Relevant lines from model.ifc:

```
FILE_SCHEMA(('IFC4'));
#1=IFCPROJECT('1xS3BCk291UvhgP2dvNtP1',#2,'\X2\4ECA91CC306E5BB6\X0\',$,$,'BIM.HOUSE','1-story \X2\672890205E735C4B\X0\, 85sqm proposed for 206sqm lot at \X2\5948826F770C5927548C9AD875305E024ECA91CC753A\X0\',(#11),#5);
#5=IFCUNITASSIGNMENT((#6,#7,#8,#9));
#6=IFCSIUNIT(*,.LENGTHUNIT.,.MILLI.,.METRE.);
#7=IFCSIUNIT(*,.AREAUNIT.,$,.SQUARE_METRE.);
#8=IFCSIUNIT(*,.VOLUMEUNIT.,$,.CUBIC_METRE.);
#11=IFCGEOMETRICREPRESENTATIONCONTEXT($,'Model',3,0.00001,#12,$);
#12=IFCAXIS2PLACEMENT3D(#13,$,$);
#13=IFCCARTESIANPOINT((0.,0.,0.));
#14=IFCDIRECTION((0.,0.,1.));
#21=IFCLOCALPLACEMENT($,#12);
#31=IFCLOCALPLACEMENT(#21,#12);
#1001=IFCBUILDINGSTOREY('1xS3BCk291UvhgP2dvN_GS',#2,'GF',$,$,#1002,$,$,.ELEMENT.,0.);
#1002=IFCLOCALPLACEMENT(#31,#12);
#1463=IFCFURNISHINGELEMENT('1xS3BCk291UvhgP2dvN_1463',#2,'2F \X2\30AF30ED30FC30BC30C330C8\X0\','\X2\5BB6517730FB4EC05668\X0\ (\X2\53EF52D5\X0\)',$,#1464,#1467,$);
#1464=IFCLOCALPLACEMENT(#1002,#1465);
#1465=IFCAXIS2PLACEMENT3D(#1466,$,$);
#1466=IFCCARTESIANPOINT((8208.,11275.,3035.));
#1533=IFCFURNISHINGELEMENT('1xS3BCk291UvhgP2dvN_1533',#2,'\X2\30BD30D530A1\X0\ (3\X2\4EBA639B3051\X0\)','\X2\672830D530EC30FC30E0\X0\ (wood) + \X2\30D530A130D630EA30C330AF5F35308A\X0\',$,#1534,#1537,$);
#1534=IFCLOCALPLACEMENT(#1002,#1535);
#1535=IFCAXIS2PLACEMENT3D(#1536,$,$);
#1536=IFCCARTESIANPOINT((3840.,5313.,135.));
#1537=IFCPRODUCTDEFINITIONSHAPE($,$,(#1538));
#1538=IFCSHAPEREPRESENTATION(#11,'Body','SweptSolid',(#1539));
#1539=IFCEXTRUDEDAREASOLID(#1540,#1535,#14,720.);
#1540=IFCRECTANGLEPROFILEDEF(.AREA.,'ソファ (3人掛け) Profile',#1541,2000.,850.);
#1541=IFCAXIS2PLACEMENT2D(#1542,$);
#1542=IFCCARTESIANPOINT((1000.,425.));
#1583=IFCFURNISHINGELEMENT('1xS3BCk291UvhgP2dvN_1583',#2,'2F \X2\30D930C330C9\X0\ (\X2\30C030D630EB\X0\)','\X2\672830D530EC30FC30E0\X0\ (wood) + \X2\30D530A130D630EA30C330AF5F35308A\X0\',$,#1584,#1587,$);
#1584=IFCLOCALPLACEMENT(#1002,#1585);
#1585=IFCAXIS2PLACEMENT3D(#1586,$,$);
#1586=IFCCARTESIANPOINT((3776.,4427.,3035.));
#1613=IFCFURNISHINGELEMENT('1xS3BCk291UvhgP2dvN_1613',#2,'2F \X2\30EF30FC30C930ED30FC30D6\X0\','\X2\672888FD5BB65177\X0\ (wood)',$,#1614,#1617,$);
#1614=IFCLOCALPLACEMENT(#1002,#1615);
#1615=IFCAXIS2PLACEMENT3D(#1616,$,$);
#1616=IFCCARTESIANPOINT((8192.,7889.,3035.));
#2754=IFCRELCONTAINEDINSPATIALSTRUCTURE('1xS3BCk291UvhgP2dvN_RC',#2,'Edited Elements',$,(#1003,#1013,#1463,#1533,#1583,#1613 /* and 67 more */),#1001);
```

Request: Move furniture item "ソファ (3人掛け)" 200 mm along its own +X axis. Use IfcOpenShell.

```python
import ifcopenshell
import ifcopenshell.api.geometry
import ifcopenshell.util.placement
import ifcopenshell.util.unit

model = ifcopenshell.open("model.ifc")
unit_scale = ifcopenshell.util.unit.calculate_unit_scale(model)

item = model.by_id(1533)
matrix = ifcopenshell.util.placement.get_local_placement(item.ObjectPlacement)
matrix[:3, 3] += matrix[:3, 0] * 0.2 / unit_scale
ifcopenshell.api.geometry.edit_object_placement(model, product=item, matrix=matrix, is_si=False)

print(ifcopenshell.util.placement.get_local_placement(item.ObjectPlacement).round(3) + 0.0)

model.write("model_v2.ifc")
```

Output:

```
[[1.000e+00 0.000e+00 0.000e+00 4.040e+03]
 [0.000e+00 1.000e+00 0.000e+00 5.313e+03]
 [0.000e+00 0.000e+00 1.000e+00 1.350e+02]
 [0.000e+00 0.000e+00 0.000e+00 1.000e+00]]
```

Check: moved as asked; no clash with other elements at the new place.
